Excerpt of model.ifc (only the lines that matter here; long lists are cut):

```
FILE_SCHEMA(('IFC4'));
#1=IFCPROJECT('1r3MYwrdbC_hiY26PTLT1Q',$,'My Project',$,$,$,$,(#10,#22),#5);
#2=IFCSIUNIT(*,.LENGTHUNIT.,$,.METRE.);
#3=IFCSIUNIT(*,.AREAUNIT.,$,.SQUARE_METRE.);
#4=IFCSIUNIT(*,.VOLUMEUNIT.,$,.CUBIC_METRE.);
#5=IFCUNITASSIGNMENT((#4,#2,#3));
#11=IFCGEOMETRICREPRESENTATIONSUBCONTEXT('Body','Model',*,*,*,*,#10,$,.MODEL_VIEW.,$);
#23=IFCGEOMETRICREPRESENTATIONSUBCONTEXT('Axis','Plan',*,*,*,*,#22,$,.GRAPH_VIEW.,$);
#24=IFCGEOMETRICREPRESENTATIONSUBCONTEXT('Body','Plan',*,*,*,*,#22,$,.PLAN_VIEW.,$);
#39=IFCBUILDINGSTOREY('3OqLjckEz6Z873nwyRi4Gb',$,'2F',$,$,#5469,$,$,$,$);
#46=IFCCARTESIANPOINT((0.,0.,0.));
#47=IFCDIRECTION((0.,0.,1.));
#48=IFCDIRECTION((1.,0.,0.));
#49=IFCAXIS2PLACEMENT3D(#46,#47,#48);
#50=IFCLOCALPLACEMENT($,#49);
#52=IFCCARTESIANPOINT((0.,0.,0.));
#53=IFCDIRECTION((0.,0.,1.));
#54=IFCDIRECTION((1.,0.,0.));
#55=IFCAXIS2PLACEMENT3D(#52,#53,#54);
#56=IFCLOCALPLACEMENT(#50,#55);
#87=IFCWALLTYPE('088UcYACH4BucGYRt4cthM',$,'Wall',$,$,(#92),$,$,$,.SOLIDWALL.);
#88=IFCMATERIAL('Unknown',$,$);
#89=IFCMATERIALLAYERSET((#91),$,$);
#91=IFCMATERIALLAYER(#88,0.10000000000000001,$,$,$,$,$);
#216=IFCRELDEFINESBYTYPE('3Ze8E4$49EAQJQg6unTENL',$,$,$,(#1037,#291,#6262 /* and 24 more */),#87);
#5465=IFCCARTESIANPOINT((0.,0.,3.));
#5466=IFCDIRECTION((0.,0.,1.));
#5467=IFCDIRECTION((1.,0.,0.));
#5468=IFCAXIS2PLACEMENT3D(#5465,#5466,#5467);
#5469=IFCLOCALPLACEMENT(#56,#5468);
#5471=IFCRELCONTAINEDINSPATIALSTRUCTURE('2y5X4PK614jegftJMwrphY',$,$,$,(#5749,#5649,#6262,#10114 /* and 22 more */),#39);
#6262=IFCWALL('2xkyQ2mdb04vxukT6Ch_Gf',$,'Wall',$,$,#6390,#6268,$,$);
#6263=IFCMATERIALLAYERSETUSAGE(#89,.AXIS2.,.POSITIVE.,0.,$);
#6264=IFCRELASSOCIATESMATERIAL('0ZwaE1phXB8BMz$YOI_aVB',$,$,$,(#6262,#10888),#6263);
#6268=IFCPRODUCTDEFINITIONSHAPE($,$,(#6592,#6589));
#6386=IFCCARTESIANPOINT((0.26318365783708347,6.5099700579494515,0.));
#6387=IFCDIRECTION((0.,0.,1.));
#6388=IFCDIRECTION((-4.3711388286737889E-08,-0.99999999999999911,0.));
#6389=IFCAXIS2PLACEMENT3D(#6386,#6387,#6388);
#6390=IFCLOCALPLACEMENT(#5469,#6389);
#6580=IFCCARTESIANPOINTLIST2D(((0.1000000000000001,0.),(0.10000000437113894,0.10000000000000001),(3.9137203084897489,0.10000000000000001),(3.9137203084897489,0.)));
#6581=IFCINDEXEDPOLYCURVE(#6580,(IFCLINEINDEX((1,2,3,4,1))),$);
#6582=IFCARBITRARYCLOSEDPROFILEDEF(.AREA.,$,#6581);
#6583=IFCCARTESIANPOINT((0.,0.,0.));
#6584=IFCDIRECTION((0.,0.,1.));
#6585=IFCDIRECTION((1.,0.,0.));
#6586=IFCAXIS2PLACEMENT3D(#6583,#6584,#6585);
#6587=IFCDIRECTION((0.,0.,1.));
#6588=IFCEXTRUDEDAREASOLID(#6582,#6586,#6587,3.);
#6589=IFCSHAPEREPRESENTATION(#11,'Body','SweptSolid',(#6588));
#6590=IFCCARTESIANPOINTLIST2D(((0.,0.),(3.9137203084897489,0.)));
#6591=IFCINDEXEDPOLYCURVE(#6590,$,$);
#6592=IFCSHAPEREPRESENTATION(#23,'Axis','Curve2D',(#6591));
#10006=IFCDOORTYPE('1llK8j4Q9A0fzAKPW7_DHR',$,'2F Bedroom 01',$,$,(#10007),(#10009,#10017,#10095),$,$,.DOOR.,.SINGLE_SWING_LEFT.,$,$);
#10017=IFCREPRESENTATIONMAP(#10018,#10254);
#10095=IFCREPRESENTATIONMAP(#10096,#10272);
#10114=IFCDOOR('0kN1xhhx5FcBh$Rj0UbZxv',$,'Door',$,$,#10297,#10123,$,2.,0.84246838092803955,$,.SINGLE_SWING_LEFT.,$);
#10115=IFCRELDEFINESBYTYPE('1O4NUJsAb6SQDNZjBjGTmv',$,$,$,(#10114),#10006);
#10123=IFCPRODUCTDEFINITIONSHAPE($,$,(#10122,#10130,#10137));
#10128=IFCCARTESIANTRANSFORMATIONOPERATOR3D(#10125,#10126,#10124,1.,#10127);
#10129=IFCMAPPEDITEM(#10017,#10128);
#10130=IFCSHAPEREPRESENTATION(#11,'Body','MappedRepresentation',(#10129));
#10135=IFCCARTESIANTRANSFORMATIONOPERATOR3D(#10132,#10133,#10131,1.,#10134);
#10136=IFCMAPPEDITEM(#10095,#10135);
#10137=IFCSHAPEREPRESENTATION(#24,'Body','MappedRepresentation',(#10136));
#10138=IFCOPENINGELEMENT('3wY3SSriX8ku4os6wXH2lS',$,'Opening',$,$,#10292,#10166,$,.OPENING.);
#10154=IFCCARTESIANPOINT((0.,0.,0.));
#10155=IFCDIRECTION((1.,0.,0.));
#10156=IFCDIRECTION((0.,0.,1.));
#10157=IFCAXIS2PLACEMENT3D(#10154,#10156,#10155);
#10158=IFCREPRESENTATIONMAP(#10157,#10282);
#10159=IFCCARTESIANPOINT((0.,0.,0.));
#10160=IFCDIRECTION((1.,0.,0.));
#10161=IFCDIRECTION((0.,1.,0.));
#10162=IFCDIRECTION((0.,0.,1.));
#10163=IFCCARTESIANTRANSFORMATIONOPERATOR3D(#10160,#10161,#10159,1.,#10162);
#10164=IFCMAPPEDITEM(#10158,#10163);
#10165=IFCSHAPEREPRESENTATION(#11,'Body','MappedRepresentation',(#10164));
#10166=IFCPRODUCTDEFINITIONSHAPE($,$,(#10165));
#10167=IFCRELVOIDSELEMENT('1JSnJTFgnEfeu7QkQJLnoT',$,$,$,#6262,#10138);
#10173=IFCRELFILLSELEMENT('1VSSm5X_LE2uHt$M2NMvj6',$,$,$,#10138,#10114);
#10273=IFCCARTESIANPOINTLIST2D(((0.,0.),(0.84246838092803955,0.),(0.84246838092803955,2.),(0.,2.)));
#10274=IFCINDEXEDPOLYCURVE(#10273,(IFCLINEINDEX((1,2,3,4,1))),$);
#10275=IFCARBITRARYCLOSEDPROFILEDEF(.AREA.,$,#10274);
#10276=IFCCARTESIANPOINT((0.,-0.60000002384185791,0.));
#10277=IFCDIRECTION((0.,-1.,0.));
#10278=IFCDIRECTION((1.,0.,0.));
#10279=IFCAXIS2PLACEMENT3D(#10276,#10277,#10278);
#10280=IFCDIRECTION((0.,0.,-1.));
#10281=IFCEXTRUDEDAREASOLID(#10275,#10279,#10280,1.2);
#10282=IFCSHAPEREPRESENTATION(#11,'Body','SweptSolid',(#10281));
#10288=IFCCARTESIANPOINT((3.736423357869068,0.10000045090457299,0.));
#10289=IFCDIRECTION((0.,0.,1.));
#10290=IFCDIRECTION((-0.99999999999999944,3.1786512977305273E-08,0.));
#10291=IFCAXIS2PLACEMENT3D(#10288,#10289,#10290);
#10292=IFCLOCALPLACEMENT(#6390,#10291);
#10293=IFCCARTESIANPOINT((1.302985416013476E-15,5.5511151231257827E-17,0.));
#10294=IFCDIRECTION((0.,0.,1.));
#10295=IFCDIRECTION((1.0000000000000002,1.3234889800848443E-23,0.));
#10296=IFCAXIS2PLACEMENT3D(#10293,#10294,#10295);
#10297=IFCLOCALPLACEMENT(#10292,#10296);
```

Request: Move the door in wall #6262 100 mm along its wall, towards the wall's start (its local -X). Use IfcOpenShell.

```python
import ifcopenshell
import ifcopenshell.api.geometry
import ifcopenshell.util.placement

model = ifcopenshell.open("model.ifc")

door = model.by_id(10114)
opening = door.FillsVoids[0].RelatingOpeningElement
wall = opening.VoidsElements[0].RelatingBuildingElement

wall_matrix = ifcopenshell.util.placement.get_local_placement(wall.ObjectPlacement)
shift = wall_matrix[:3, 0] * -0.1
before = ifcopenshell.util.placement.get_local_placement(door.ObjectPlacement)[:3, 3].copy()

# The door is placed relative to its opening, so it follows when the opening moves.
matrix = ifcopenshell.util.placement.get_local_placement(opening.ObjectPlacement)
matrix[:3, 3] += shift
ifcopenshell.api.geometry.edit_object_placement(
    model, product=opening, matrix=matrix, is_si=False, should_transform_children=True
)

after = ifcopenshell.util.placement.get_local_placement(door.ObjectPlacement)[:3, 3]
print("door moved by", (after - before).round(3) + 0.0)

model.write("model_v2.ifc")
```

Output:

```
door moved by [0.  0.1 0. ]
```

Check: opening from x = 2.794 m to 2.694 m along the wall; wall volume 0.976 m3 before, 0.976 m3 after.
